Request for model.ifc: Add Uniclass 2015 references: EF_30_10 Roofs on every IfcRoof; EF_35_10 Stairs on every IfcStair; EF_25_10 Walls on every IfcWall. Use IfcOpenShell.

First a look at what the model holds.

```python
import ifcopenshell

model = ifcopenshell.open("model.ifc")
print(model.schema)
print("classifications:", [c.Name for c in model.by_type("IfcClassification")])
for ifc_class in ("IfcDoor", "IfcRoof", "IfcStair", "IfcWall", "IfcWindow"):
    print(ifc_class, len(model.by_type(ifc_class)))
```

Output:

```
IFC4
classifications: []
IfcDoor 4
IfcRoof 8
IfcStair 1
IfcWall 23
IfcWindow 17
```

```python
import ifcopenshell
import ifcopenshell.api.classification

model = ifcopenshell.open("model.ifc")

system = ifcopenshell.api.classification.add_classification(model, classification="Uniclass 2015")

codes = {
    "IfcRoof": ("EF_30_10", "Roofs"),
    "IfcStair": ("EF_35_10", "Stairs"),
    "IfcWall": ("EF_25_10", "Walls"),
}
for ifc_class, (code, name) in codes.items():
    products = model.by_type(ifc_class)
    ifcopenshell.api.classification.add_reference(
        model, products=products, classification=system, identification=code, name=name
    )
    print(code, len(products))

model.write("model_rev.ifc")
```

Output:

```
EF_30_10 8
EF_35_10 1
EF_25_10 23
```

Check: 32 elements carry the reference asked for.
